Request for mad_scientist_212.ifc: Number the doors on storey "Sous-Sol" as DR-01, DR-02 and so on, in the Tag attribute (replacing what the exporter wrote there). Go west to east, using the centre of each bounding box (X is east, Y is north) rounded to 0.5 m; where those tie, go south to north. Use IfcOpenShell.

First a look at what the model holds.

```python
import ifcopenshell
import ifcopenshell.util.element
import ifcopenshell.util.placement

model = ifcopenshell.open("mad_scientist_212.ifc")
print(model.schema)
storey = next(s for s in model.by_type("IfcBuildingStorey") if s.Name == "Sous-Sol")
doors = [e for e in ifcopenshell.util.element.get_decomposition(storey) if e.is_a("IfcDoor")]
for e in sorted(doors, key=lambda e: e.id()):
    origin = ifcopenshell.util.placement.get_local_placement(e.ObjectPlacement)[:3, 3]
    print(e.id(), e.Tag, e.Name, origin.round(2) + 0.0, sep=" | ")
```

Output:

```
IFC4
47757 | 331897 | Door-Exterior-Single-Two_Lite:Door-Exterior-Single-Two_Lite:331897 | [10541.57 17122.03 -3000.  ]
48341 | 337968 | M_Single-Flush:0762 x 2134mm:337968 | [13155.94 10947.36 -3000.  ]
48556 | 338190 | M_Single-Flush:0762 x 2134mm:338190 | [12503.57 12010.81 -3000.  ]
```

```python
import ifcopenshell
import ifcopenshell.geom
import ifcopenshell.util.element
import ifcopenshell.util.shape

model = ifcopenshell.open("mad_scientist_212.ifc")
settings = ifcopenshell.geom.settings()
settings.set("use-world-coords", True)


def centre(element):
    shape = ifcopenshell.geom.create_shape(settings, element)
    return ifcopenshell.util.shape.get_bbox_centroid(shape.geometry)


storey = next(s for s in model.by_type("IfcBuildingStorey") if s.Name == "Sous-Sol")
doors = [e for e in ifcopenshell.util.element.get_decomposition(storey) if e.is_a("IfcDoor")]

# Insertion points can sit at a corner or the storey origin, so sort by the geometry (in metres).
centres = {e: centre(e) for e in doors}
doors.sort(key=lambda e: (round(centres[e][0] / 0.5), centres[e][1]))

for i, e in enumerate(doors, start=1):
    number = f"DR-{i:02d}"
    e.Tag = number
    print(e.id(), number)

model.write("mad_scientist_212_updated.ifc")
```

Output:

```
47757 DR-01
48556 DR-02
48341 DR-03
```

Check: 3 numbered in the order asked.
